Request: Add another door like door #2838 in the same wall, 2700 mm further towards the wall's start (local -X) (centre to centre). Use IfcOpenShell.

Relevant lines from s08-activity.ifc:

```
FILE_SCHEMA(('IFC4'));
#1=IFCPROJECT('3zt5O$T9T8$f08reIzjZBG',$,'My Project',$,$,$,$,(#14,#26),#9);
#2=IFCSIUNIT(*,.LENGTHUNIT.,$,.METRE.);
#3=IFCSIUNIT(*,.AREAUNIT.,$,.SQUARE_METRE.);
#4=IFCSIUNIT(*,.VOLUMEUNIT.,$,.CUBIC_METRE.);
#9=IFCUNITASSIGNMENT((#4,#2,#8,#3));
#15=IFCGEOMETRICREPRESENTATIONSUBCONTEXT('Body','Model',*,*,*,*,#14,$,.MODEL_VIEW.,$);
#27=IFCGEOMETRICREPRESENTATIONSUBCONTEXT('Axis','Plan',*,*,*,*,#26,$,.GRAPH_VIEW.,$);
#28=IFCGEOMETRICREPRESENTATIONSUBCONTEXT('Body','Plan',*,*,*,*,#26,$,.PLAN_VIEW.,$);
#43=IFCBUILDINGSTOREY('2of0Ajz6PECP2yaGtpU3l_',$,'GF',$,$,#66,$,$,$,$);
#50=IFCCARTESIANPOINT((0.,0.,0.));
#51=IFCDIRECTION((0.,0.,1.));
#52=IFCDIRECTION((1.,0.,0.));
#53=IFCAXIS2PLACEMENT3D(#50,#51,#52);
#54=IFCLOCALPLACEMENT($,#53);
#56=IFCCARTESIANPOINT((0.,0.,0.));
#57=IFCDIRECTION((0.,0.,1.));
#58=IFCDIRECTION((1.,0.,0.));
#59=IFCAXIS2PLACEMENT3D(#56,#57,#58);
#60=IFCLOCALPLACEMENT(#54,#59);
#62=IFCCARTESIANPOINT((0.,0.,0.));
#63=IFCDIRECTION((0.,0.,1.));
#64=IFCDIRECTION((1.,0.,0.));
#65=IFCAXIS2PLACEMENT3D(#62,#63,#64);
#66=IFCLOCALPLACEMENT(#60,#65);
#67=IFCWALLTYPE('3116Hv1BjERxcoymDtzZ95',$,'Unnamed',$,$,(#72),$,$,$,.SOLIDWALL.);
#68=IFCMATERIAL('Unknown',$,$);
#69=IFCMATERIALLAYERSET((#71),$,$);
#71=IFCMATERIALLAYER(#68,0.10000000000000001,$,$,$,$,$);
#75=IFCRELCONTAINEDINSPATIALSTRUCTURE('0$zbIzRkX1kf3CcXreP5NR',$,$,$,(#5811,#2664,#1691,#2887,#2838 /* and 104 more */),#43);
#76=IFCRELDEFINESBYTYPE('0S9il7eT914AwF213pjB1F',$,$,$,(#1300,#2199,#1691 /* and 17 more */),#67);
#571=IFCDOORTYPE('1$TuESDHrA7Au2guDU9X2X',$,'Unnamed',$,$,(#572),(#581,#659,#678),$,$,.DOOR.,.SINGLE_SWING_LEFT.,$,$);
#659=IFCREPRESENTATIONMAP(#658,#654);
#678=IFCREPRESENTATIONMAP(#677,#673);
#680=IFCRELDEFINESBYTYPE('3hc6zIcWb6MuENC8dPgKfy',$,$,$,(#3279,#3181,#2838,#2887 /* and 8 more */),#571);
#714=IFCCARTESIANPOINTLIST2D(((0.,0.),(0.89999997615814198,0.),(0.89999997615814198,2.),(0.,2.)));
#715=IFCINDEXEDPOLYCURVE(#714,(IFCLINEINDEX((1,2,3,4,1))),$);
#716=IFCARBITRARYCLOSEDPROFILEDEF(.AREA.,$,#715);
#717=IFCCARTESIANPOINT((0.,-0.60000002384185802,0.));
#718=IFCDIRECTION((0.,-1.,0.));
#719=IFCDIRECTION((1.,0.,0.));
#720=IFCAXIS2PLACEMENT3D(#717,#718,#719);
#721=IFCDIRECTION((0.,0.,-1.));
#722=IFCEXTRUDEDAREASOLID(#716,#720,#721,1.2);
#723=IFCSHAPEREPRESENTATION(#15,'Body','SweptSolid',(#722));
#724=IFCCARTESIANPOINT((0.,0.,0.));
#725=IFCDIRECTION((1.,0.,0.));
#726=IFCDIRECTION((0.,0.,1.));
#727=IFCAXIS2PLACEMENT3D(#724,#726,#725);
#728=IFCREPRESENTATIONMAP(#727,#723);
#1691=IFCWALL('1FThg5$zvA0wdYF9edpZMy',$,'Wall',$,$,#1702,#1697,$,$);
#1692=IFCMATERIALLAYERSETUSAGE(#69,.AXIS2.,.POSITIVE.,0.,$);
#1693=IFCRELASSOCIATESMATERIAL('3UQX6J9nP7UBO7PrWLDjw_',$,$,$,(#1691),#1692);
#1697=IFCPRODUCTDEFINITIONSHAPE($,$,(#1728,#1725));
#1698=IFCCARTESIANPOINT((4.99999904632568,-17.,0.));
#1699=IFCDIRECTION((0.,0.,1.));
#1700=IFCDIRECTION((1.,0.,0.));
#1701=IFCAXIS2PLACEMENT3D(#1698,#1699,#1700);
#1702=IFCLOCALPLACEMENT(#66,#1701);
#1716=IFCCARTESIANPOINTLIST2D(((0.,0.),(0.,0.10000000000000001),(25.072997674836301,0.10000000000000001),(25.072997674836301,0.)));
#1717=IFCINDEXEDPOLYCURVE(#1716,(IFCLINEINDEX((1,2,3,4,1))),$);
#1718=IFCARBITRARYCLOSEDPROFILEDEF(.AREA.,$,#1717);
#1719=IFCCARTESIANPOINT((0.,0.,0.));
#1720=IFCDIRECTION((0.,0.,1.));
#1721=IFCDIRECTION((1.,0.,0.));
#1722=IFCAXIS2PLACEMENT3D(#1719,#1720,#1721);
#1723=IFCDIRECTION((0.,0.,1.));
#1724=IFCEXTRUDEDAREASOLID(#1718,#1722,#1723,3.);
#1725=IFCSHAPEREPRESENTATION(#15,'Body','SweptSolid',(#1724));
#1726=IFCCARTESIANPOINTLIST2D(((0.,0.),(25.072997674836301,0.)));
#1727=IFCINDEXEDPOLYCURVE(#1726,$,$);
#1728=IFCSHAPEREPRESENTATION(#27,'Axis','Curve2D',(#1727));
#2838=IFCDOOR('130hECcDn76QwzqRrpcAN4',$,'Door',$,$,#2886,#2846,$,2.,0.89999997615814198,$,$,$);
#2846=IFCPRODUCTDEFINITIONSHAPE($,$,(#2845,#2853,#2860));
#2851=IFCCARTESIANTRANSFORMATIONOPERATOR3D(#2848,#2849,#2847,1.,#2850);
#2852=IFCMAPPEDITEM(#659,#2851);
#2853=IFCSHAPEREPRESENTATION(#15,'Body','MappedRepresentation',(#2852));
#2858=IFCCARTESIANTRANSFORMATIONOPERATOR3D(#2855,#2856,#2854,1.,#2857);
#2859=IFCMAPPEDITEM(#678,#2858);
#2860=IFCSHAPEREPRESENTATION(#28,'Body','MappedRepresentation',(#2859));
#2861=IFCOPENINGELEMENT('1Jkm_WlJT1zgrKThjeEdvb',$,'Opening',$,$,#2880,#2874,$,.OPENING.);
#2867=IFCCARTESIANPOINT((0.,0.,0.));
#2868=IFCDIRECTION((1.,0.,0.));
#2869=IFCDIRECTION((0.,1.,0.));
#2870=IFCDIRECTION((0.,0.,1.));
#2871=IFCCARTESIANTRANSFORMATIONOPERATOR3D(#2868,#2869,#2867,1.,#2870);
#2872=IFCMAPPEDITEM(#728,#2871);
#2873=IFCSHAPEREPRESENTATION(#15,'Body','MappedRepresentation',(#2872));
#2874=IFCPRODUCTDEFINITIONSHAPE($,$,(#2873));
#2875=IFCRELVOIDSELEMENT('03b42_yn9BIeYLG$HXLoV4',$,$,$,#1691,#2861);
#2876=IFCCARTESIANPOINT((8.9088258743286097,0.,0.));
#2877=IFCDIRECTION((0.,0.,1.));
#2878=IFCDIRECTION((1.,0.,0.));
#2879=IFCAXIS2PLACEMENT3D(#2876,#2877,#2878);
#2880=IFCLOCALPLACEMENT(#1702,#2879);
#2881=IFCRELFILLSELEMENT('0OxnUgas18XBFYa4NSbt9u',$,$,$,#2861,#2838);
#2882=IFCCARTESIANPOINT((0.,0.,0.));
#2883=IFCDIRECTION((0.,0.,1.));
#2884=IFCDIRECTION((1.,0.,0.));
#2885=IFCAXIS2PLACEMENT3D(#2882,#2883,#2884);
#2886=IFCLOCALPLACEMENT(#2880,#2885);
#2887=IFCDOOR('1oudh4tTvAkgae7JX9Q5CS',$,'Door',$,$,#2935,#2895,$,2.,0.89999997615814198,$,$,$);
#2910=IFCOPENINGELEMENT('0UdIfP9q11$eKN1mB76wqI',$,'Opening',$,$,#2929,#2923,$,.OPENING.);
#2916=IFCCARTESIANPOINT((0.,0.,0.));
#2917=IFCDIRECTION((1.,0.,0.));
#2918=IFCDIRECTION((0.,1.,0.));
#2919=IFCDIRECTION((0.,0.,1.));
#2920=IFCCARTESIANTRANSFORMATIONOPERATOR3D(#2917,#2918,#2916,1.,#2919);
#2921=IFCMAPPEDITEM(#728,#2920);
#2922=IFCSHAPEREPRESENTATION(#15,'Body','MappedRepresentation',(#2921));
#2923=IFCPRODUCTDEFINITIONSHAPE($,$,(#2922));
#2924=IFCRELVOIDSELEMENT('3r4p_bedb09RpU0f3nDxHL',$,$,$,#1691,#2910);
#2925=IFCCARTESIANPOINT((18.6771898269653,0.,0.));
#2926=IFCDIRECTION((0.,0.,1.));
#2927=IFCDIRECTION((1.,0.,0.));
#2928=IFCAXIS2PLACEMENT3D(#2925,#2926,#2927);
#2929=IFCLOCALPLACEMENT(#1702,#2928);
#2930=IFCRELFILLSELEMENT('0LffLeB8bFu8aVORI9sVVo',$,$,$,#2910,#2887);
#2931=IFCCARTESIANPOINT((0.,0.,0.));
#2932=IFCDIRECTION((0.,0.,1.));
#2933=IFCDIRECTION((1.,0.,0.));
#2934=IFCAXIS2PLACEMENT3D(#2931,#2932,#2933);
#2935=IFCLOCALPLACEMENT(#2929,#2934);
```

```python
import ifcopenshell
import ifcopenshell.api.feature
import ifcopenshell.api.geometry
import ifcopenshell.api.root
import ifcopenshell.geom
import ifcopenshell.util.element
import ifcopenshell.util.placement
import ifcopenshell.util.shape

model = ifcopenshell.open("s08-activity.ifc")
settings = ifcopenshell.geom.settings()


def volume(element):
    """Net volume in cubic metres, openings subtracted."""
    shape = ifcopenshell.geom.create_shape(settings, element)
    return ifcopenshell.util.shape.get_volume(shape.geometry)


door = model.by_guid("130hECcDn76QwzqRrpcAN4")
opening = door.FillsVoids[0].RelatingOpeningElement
wall = opening.VoidsElements[0].RelatingBuildingElement
before = volume(wall)
shift = ifcopenshell.util.placement.get_local_placement(wall.ObjectPlacement)[:3, 0] * -2.7

# copy_class copies the void relationship, type, container and properties, but no geometry.
new_opening = ifcopenshell.api.root.copy_class(model, product=opening)
new_opening.Representation = ifcopenshell.util.element.copy_deep(
    model, opening.Representation, exclude=["IfcGeometricRepresentationContext", "IfcRepresentationMap"]
)
new_door = ifcopenshell.api.root.copy_class(model, product=door)
new_door.Representation = ifcopenshell.util.element.copy_deep(
    model, door.Representation, exclude=["IfcGeometricRepresentationContext", "IfcRepresentationMap"]
)
ifcopenshell.api.feature.add_filling(model, opening=new_opening, element=new_door)

for old, new in ((opening, new_opening), (door, new_door)):
    matrix = ifcopenshell.util.placement.get_local_placement(old.ObjectPlacement)
    matrix[:3, 3] += shift
    ifcopenshell.api.geometry.edit_object_placement(model, product=new, matrix=matrix, is_si=False)

after = volume(wall)

print(f"wall volume {before:.3f} -> {after:.3f} m3")

model.write("s08-activity_rev.ifc")
```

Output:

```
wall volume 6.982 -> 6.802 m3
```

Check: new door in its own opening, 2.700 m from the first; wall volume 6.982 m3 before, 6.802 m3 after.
